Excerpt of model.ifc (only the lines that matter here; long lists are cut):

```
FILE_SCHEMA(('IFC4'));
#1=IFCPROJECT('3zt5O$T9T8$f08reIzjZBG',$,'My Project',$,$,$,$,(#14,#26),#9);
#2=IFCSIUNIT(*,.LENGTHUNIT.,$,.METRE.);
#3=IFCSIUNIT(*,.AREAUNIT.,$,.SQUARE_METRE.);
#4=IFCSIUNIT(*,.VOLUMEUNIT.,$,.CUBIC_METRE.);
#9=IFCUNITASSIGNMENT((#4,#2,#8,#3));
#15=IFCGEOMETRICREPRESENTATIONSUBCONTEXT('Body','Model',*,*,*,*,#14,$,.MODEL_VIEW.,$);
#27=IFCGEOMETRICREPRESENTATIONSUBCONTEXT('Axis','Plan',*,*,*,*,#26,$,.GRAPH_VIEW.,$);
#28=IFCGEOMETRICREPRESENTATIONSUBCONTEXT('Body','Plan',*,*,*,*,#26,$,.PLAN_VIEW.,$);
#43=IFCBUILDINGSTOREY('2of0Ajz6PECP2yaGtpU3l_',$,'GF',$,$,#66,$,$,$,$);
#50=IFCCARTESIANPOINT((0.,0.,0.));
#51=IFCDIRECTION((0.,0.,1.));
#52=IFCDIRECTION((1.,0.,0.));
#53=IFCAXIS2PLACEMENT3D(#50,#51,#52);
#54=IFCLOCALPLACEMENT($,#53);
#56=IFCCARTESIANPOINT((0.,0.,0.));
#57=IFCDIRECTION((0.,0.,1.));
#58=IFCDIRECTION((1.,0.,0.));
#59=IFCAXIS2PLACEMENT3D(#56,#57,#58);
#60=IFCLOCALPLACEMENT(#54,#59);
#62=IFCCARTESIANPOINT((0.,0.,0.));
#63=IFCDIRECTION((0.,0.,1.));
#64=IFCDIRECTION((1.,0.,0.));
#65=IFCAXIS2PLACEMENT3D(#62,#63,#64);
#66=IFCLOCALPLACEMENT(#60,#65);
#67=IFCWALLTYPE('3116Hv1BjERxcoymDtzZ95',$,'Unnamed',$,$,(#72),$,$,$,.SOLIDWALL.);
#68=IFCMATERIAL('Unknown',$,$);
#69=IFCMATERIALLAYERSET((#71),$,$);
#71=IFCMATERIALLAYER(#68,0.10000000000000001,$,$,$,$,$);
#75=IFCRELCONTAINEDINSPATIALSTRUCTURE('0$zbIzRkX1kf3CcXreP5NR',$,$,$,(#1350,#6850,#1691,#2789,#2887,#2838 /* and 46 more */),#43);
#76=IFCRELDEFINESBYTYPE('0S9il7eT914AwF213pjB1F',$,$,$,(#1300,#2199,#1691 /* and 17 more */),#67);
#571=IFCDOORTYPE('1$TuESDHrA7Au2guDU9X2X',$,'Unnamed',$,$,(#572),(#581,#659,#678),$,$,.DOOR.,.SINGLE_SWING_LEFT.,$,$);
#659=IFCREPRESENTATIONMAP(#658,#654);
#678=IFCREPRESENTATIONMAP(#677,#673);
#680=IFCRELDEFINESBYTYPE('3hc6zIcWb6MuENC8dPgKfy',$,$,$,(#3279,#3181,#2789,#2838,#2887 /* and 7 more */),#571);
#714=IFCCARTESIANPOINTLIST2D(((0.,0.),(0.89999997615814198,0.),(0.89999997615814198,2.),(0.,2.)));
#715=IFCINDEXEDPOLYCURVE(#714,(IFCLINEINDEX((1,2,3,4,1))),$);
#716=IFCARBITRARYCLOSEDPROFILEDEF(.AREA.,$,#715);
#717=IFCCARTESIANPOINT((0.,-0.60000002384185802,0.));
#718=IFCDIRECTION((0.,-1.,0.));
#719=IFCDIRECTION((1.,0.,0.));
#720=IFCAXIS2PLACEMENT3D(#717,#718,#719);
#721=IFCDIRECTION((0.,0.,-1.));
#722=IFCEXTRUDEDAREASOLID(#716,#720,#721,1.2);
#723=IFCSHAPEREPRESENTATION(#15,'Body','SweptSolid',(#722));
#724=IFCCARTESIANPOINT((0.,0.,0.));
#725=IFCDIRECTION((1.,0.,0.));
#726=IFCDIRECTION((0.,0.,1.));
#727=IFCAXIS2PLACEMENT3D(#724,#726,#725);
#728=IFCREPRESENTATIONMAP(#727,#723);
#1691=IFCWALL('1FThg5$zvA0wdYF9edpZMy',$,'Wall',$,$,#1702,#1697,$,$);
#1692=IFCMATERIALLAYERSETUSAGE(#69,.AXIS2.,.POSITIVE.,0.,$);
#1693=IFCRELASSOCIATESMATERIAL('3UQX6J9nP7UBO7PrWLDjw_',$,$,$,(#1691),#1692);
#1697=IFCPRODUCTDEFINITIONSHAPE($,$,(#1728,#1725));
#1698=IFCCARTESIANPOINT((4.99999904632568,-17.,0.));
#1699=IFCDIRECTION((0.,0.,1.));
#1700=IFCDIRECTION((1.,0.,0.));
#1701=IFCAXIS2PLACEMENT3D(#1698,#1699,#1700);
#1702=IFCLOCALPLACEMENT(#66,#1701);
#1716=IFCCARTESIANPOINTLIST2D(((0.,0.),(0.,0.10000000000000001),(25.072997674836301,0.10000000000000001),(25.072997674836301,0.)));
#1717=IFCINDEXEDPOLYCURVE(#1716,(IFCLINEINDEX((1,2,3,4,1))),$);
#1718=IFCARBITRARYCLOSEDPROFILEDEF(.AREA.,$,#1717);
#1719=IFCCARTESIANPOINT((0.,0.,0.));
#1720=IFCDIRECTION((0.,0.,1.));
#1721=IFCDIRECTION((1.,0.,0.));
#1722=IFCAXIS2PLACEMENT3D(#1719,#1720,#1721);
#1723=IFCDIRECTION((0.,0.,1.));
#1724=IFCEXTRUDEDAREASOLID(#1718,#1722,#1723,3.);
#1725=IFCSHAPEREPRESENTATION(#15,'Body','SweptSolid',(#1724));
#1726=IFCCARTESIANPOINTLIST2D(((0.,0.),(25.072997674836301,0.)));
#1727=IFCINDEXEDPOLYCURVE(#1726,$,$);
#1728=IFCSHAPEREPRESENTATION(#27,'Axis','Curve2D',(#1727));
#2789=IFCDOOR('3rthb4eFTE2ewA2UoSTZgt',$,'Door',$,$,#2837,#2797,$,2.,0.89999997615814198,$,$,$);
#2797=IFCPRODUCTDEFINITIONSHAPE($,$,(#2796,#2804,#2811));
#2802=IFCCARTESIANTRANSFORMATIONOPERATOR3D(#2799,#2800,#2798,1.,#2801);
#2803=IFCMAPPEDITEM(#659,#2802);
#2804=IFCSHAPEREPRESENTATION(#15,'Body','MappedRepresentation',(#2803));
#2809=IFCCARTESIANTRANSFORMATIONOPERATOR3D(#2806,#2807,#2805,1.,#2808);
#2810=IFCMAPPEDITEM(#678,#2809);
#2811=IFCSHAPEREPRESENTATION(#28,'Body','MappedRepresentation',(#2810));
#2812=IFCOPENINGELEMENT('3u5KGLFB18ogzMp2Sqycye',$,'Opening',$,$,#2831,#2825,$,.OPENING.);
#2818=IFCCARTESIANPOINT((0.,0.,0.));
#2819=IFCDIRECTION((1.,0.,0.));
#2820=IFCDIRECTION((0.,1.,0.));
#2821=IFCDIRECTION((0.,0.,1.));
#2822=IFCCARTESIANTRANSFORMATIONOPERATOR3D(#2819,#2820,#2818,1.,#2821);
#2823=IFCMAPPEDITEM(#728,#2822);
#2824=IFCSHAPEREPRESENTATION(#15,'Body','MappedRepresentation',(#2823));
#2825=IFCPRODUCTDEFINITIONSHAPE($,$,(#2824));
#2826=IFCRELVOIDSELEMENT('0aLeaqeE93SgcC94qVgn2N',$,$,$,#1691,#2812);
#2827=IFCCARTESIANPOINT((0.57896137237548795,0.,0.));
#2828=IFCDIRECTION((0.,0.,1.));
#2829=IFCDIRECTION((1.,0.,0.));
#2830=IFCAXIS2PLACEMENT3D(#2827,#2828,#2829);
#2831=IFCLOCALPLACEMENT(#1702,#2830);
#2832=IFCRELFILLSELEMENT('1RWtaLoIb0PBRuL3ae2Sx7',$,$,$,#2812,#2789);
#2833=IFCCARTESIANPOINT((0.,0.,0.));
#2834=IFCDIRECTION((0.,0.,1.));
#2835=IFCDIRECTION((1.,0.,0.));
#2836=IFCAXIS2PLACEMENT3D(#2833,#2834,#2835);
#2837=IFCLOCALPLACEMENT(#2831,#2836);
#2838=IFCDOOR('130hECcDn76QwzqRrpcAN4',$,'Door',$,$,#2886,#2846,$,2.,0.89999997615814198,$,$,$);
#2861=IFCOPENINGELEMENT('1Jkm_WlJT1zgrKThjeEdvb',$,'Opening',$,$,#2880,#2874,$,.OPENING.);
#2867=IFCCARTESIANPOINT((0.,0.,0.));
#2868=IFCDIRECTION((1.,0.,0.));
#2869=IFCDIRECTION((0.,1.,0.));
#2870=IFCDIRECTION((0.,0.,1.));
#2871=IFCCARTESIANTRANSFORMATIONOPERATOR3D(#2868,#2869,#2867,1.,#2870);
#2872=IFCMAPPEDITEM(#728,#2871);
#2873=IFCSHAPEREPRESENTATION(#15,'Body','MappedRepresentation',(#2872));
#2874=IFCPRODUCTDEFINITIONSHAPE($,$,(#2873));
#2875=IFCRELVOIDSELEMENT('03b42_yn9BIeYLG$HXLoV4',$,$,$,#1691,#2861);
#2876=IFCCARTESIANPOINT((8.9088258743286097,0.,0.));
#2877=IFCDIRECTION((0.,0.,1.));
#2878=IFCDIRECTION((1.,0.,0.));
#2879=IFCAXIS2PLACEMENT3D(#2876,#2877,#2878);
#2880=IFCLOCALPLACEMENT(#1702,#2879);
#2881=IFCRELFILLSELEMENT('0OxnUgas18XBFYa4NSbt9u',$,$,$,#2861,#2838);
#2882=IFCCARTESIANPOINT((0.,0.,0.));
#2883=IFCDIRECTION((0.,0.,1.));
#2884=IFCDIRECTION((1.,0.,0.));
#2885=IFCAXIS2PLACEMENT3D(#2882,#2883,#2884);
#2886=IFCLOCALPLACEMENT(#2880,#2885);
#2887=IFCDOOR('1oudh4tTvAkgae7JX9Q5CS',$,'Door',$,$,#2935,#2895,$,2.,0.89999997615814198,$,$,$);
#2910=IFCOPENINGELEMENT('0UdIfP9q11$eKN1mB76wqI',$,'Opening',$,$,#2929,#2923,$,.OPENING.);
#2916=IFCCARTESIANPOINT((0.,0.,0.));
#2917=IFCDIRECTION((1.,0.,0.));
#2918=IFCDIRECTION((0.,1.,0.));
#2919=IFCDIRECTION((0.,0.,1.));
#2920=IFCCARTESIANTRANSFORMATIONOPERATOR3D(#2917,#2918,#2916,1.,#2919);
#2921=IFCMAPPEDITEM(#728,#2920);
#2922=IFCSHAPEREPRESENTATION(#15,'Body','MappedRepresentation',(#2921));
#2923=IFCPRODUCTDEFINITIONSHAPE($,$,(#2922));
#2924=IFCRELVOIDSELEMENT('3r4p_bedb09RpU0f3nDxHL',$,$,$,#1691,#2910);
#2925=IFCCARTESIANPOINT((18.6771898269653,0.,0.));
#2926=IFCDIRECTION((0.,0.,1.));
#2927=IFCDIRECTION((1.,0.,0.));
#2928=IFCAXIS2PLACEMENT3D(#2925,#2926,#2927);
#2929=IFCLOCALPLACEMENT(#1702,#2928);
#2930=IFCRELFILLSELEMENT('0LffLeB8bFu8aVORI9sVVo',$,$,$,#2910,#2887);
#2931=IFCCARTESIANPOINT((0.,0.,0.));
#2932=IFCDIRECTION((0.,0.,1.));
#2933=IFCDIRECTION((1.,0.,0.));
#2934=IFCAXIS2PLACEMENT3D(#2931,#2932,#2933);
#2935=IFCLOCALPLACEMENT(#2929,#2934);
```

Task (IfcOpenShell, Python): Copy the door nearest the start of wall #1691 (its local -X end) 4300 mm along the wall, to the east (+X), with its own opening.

```python
import ifcopenshell
import ifcopenshell.api.feature
import ifcopenshell.api.geometry
import ifcopenshell.api.root
import ifcopenshell.geom
import ifcopenshell.util.element
import ifcopenshell.util.placement
import ifcopenshell.util.shape

model = ifcopenshell.open("model.ifc")
settings = ifcopenshell.geom.settings()


def volume(element):
    """Net volume in cubic metres, openings subtracted."""
    shape = ifcopenshell.geom.create_shape(settings, element)
    return ifcopenshell.util.shape.get_volume(shape.geometry)


door = model.by_guid("3rthb4eFTE2ewA2UoSTZgt")
opening = door.FillsVoids[0].RelatingOpeningElement
wall = opening.VoidsElements[0].RelatingBuildingElement
before = volume(wall)
shift = ifcopenshell.util.placement.get_local_placement(wall.ObjectPlacement)[:3, 0] * 4.3

# copy_class copies the void relationship, type, container and properties, but no geometry.
new_opening = ifcopenshell.api.root.copy_class(model, product=opening)
new_opening.Representation = ifcopenshell.util.element.copy_deep(
    model, opening.Representation, exclude=["IfcGeometricRepresentationContext", "IfcRepresentationMap"]
)
new_door = ifcopenshell.api.root.copy_class(model, product=door)
new_door.Representation = ifcopenshell.util.element.copy_deep(
    model, door.Representation, exclude=["IfcGeometricRepresentationContext", "IfcRepresentationMap"]
)
ifcopenshell.api.feature.add_filling(model, opening=new_opening, element=new_door)

for old, new in ((opening, new_opening), (door, new_door)):
    matrix = ifcopenshell.util.placement.get_local_placement(old.ObjectPlacement)
    matrix[:3, 3] += shift
    ifcopenshell.api.geometry.edit_object_placement(model, product=new, matrix=matrix, is_si=False)

after = volume(wall)

print(f"wall volume {before:.3f} -> {after:.3f} m3")

model.write("model_rev.ifc")
```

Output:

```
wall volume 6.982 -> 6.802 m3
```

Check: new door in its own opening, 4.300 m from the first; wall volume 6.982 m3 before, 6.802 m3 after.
